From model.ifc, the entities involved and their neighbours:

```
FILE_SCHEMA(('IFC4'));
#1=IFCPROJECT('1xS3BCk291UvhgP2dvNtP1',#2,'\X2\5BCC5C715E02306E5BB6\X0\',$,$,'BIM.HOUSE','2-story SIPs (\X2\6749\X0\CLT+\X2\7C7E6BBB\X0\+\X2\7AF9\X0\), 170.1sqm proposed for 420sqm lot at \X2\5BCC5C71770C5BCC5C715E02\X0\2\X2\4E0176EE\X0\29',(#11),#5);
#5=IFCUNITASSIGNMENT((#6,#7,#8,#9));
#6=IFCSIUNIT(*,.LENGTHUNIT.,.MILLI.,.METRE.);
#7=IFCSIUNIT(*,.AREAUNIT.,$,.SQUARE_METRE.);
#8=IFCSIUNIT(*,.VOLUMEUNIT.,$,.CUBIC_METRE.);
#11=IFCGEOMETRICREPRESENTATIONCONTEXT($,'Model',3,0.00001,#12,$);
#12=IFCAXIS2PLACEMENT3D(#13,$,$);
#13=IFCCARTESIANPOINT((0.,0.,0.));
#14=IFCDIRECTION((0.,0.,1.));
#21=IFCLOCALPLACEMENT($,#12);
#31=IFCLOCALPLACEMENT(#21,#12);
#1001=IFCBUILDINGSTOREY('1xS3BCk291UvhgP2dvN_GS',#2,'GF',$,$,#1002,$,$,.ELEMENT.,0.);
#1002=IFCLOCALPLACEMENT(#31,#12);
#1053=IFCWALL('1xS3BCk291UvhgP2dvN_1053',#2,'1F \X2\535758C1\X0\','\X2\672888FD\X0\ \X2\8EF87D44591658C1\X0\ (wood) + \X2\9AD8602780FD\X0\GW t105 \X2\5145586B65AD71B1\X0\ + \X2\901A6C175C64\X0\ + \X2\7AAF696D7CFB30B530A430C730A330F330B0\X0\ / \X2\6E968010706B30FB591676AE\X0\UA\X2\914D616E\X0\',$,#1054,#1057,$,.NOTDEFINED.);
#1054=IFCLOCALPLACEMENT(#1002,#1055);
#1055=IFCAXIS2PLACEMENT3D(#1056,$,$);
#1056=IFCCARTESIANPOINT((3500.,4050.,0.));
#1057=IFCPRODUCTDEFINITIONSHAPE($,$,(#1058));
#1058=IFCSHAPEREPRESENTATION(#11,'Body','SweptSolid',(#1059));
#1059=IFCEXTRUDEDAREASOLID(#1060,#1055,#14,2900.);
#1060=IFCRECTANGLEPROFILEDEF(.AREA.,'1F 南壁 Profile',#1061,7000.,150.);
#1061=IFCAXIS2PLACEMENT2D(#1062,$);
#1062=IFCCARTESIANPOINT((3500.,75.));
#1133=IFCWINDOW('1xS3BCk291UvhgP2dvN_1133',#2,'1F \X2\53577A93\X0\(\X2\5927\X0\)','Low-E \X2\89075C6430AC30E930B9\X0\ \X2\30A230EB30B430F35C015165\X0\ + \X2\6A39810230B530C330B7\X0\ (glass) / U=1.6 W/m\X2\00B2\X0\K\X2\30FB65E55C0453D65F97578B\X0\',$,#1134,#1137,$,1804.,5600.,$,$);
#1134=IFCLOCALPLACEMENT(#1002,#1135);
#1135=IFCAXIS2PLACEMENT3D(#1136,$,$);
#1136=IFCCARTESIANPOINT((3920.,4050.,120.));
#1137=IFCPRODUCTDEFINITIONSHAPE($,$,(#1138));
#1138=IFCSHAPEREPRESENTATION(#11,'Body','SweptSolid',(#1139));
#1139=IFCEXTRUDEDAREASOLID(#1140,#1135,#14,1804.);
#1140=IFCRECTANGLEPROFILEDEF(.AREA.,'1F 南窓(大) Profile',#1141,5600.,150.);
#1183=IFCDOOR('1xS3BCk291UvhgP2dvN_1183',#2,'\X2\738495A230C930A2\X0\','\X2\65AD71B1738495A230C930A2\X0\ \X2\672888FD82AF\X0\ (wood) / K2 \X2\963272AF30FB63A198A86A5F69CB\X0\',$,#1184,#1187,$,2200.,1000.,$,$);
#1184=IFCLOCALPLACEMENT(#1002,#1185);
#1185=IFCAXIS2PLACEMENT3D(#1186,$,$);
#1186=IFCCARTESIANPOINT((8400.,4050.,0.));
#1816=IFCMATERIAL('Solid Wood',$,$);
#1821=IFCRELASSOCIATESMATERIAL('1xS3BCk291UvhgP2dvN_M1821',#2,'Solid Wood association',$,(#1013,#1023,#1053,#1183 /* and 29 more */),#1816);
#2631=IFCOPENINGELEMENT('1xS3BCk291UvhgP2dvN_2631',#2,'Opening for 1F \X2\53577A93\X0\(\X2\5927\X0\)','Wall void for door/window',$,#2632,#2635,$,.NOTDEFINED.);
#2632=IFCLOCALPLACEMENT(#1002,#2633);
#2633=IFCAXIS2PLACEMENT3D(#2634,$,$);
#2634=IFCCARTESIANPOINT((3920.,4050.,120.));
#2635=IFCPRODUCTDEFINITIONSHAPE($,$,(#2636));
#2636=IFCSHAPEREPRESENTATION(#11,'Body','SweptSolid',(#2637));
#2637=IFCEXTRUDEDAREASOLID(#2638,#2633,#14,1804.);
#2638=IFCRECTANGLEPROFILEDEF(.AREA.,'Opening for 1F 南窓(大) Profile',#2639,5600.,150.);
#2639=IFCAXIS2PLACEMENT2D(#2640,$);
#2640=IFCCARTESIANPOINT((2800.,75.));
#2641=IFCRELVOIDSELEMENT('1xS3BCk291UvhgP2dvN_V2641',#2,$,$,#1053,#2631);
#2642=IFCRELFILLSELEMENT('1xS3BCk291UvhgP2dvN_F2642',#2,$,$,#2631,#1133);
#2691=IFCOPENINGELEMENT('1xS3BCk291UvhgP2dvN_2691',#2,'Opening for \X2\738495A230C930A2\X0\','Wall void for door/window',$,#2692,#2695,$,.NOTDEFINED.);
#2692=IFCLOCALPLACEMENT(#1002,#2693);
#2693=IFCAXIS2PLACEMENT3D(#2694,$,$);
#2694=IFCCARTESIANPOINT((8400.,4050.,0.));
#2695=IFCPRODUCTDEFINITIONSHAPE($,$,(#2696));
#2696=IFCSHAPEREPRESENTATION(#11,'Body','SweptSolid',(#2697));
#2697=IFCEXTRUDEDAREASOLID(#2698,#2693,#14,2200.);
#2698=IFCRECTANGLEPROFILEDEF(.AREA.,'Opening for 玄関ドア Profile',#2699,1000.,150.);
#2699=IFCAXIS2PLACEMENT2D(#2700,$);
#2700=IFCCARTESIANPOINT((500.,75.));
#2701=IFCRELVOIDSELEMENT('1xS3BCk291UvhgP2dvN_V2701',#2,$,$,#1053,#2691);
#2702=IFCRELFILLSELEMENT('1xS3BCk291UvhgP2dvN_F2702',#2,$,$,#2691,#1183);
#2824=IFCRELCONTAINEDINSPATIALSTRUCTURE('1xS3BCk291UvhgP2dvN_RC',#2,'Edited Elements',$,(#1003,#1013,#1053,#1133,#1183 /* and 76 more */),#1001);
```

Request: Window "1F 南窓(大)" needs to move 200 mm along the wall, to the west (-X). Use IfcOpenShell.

```python
import ifcopenshell
import ifcopenshell.api.geometry
import ifcopenshell.util.placement

model = ifcopenshell.open("model.ifc")

window = model.by_guid("1xS3BCk291UvhgP2dvN_1133")
opening = window.FillsVoids[0].RelatingOpeningElement
wall = opening.VoidsElements[0].RelatingBuildingElement

wall_matrix = ifcopenshell.util.placement.get_local_placement(wall.ObjectPlacement)
shift = wall_matrix[:3, 0] * -200.0
before = ifcopenshell.util.placement.get_local_placement(window.ObjectPlacement)[:3, 3].copy()

# The window is not placed relative to its opening, so move both.
for product in (opening, window):
    matrix = ifcopenshell.util.placement.get_local_placement(product.ObjectPlacement)
    matrix[:3, 3] += shift
    ifcopenshell.api.geometry.edit_object_placement(model, product=product, matrix=matrix, is_si=False)

after = ifcopenshell.util.placement.get_local_placement(window.ObjectPlacement)[:3, 3]
print("window moved by", (after - before).round(3) + 0.0)

model.write("model_updated.ifc")
```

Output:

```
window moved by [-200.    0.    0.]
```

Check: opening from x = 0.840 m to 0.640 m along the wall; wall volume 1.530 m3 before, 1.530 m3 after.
